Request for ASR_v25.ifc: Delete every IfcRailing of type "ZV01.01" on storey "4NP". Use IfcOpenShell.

First a look at what the model holds.

```python
import ifcopenshell
import ifcopenshell.util.element

model = ifcopenshell.open("ASR_v25.ifc")
print(model.schema)
storey = next(s for s in model.by_type("IfcBuildingStorey") if s.Name == "4NP")
railings = [e for e in ifcopenshell.util.element.get_decomposition(storey) if e.is_a("IfcRailing")]
seen = {}
for e in railings:
    element_type = ifcopenshell.util.element.get_type(e)
    name = element_type.Name if element_type not in (None, e) else None
    seen[name] = seen.get(name, 0) + 1
for name, count in sorted(seen.items(), key=str):
    print(count, "x", name)
```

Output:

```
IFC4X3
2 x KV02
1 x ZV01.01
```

```python
import ifcopenshell
import ifcopenshell.api.root
import ifcopenshell.util.element

model = ifcopenshell.open("ASR_v25.ifc")

storey = next(s for s in model.by_type("IfcBuildingStorey") if s.Name == "4NP")
railings = [e for e in ifcopenshell.util.element.get_decomposition(storey) if e.is_a("IfcRailing")]
targets = [e for e in railings if (t := ifcopenshell.util.element.get_type(e)) not in (None, e) and t.Name == "ZV01.01"]

for e in targets:
    ifcopenshell.api.root.remove_product(model, product=e)
print(len(targets), "removed")

model.write("ASR_v25_rev.ifc")
```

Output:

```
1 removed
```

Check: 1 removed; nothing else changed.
